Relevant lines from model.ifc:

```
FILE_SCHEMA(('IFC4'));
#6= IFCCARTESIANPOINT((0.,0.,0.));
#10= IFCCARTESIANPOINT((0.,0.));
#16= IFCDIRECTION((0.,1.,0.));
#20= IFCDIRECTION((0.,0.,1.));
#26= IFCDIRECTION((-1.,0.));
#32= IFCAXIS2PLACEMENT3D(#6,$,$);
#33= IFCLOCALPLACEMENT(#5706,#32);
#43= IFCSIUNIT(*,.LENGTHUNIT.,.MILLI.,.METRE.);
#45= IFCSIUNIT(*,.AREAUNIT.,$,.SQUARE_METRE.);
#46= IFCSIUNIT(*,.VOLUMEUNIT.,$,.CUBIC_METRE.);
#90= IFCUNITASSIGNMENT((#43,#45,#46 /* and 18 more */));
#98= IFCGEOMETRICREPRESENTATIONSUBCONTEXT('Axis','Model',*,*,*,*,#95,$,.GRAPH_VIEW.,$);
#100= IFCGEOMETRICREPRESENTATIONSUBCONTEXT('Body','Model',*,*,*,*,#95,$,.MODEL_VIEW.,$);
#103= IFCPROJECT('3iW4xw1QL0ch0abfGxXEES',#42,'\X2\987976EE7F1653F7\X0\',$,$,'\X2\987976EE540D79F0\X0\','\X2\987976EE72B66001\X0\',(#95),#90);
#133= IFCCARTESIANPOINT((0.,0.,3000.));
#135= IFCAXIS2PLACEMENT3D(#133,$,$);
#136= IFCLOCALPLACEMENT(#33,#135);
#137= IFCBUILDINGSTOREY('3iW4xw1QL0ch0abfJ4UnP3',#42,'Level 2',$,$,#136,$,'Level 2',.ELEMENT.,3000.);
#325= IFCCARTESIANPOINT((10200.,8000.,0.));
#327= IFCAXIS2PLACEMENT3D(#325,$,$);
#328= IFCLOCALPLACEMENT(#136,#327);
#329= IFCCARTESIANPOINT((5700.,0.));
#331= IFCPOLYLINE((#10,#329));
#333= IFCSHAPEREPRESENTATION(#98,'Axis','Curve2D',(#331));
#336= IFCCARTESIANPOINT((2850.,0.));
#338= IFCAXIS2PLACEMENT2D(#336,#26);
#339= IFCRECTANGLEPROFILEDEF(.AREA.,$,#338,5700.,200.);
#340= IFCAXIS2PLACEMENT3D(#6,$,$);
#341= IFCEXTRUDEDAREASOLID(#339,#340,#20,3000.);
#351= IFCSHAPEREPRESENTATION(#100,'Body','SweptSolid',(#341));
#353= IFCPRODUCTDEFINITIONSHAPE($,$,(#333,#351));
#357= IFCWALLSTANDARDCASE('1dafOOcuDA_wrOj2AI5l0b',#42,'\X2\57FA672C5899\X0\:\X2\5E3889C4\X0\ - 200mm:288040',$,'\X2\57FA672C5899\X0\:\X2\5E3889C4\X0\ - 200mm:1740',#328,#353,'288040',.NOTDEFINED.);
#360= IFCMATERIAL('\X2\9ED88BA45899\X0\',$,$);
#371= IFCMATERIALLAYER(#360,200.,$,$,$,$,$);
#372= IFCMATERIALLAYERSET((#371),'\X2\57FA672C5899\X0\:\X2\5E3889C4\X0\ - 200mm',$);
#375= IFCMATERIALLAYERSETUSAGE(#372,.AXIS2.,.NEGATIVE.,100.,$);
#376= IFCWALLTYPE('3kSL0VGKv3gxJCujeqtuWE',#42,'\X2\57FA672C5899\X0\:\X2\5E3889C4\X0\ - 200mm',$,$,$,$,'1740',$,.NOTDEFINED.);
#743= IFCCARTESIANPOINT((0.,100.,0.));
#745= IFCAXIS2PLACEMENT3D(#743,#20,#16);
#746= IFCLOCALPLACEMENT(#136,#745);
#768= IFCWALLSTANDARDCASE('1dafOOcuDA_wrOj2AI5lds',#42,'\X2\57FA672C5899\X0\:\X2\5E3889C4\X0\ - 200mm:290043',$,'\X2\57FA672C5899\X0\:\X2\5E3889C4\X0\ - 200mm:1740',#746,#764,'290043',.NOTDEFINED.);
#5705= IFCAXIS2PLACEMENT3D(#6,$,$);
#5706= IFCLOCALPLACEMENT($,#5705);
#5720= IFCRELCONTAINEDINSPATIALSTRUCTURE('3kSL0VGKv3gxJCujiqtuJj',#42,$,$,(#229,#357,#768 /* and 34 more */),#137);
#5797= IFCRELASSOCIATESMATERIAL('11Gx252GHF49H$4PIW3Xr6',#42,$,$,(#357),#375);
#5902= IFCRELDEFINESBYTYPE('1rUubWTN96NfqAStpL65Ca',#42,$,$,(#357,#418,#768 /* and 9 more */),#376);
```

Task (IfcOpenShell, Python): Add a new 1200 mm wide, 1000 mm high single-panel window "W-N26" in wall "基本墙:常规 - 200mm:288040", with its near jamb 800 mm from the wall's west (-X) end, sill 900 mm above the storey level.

```python
import numpy as np
import ifcopenshell
import ifcopenshell.api.feature
import ifcopenshell.api.geometry
import ifcopenshell.api.root
import ifcopenshell.api.spatial
import ifcopenshell.geom
import ifcopenshell.util.element
import ifcopenshell.util.placement
import ifcopenshell.util.representation
import ifcopenshell.util.shape
import ifcopenshell.util.unit

model = ifcopenshell.open("model.ifc")
unit_scale = ifcopenshell.util.unit.calculate_unit_scale(model)
settings = ifcopenshell.geom.settings()


def volume(element):
    """Net volume in cubic metres, openings subtracted."""
    shape = ifcopenshell.geom.create_shape(settings, element)
    return ifcopenshell.util.shape.get_volume(shape.geometry)


wall = model.by_guid("1dafOOcuDA_wrOj2AI5l0b")
storey = ifcopenshell.util.element.get_container(wall, ifc_class="IfcBuildingStorey")
context = ifcopenshell.util.representation.get_context(model, "Model", "Body", "MODEL_VIEW")
before = volume(wall)

width, height, from_end, sill = 1.2, 1, 0.8, 0.9  # metres

# The wall runs along its own X axis, and the end named is its -X end.
wall_shape = ifcopenshell.geom.create_shape(settings, wall)
x, y, z = ifcopenshell.util.shape.get_vertices(wall_shape.geometry).T
start = x.min() + from_end
face, thickness = float(y.min()), float(y.max() - y.min())
wall_matrix = ifcopenshell.util.placement.get_local_placement(wall.ObjectPlacement)
level = ifcopenshell.util.placement.get_local_placement(storey.ObjectPlacement)[2, 3]


def in_wall(x, y):
    """Placement at x, y metres in the wall's axes, at sill height."""
    matrix = wall_matrix.copy()
    matrix[:, 3] = wall_matrix @ np.array([x / unit_scale, y / unit_scale, 0.0, 1.0])
    matrix[2, 3] = level + sill / unit_scale
    return matrix


# Opening: a box that overshoots both wall faces by 50 mm.
opening = ifcopenshell.api.root.create_entity(model, ifc_class="IfcOpeningElement", predefined_type="OPENING")
box = ifcopenshell.api.geometry.add_wall_representation(
    model, context=context, length=width, height=height, thickness=thickness + 0.1
)
ifcopenshell.api.geometry.assign_representation(model, product=opening, representation=box)
ifcopenshell.api.geometry.edit_object_placement(model, product=opening, matrix=in_wall(start, face - 0.05), is_si=False)
ifcopenshell.api.feature.add_feature(model, feature=opening, element=wall)

window = ifcopenshell.api.root.create_entity(model, ifc_class="IfcWindow", name="W-N26", predefined_type="WINDOW")
window.OverallWidth, window.OverallHeight = width / unit_scale, height / unit_scale
window.PartitioningType = "SINGLE_PANEL"
body = ifcopenshell.api.geometry.add_window_representation(
    model,
    context=context,
    overall_width=window.OverallWidth,
    overall_height=window.OverallHeight,
    partition_type="SINGLE_PANEL",
)
ifcopenshell.api.geometry.assign_representation(model, product=window, representation=body)
ifcopenshell.api.spatial.assign_container(model, products=[window], relating_structure=storey)
ifcopenshell.api.feature.add_filling(model, opening=opening, element=window)

# Centre the window in the wall's thickness.
ifcopenshell.api.geometry.edit_object_placement(model, product=window, matrix=in_wall(start, face), is_si=False)
window_shape = ifcopenshell.geom.create_shape(settings, window)
depth = ifcopenshell.util.shape.get_vertices(window_shape.geometry)[:, 1]
offset = face + thickness / 2 - (depth.min() + depth.max()) / 2
ifcopenshell.api.geometry.edit_object_placement(model, product=window, matrix=in_wall(start, offset), is_si=False)

after = volume(wall)

print(f"wall volume {before:.3f} -> {after:.3f} m3")

model.write("model_rev.ifc")
```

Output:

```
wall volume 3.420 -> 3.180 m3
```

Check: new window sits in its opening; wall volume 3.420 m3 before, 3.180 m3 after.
